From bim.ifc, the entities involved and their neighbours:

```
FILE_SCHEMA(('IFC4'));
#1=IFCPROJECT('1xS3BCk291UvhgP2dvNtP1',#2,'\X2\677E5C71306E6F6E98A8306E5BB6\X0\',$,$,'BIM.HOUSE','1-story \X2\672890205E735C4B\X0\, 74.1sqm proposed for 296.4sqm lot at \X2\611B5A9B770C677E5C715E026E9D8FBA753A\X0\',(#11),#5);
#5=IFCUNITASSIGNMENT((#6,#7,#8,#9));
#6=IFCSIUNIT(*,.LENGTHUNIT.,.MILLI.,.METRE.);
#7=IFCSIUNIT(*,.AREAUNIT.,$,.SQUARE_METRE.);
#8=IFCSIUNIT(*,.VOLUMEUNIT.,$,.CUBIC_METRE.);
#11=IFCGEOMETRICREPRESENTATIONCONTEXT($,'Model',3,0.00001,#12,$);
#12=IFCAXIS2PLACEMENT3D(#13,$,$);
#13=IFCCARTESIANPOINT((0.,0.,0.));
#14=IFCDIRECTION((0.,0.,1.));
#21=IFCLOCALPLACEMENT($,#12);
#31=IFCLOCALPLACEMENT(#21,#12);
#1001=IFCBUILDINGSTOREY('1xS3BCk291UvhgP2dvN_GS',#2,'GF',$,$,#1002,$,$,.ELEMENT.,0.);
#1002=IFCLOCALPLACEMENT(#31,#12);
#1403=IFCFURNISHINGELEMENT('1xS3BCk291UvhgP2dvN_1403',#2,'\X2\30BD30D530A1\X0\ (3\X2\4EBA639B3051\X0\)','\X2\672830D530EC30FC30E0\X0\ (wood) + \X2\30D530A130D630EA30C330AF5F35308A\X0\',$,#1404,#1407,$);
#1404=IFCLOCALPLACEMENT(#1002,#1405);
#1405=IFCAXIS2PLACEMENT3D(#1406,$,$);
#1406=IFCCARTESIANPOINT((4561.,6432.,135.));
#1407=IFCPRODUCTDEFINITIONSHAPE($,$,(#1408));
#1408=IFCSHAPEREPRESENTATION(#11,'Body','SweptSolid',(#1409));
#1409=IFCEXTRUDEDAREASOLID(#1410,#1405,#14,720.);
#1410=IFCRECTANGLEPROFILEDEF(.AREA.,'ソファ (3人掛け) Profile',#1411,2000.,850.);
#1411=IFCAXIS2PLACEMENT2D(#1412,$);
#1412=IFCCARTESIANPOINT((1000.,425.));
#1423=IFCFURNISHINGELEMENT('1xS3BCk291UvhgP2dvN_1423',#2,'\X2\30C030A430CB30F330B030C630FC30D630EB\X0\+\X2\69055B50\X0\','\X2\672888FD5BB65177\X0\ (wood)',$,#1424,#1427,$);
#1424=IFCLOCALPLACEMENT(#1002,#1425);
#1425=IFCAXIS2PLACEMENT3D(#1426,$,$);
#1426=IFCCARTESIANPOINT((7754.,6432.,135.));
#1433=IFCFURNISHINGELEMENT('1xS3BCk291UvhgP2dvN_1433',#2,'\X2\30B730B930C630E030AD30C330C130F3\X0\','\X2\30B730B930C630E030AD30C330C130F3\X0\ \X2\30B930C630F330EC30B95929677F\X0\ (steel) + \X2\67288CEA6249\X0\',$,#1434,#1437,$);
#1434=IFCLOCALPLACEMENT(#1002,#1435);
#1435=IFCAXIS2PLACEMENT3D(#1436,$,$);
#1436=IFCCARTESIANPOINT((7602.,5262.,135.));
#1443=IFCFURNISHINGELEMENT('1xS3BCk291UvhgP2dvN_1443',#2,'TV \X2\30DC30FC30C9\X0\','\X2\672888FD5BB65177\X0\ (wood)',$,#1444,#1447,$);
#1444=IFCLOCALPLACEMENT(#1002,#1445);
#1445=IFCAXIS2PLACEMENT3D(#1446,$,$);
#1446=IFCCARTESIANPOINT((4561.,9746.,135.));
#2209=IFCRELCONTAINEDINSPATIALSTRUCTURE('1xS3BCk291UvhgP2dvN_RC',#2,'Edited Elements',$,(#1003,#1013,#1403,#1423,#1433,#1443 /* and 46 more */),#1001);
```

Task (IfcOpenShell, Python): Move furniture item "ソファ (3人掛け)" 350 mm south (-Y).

```python
import ifcopenshell
import ifcopenshell.api.geometry
import ifcopenshell.util.placement
import ifcopenshell.util.unit

model = ifcopenshell.open("bim.ifc")
unit_scale = ifcopenshell.util.unit.calculate_unit_scale(model)

item = model.by_id(1403)
matrix = ifcopenshell.util.placement.get_local_placement(item.ObjectPlacement)
matrix[1, 3] -= 0.35 / unit_scale
ifcopenshell.api.geometry.edit_object_placement(model, product=item, matrix=matrix, is_si=False)

print(ifcopenshell.util.placement.get_local_placement(item.ObjectPlacement).round(3) + 0.0)

model.write("bim-out.ifc")
```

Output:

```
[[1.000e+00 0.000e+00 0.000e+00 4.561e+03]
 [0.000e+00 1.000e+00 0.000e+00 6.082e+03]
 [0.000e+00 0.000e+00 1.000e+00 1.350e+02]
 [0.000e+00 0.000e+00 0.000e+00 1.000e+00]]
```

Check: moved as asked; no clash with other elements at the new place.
